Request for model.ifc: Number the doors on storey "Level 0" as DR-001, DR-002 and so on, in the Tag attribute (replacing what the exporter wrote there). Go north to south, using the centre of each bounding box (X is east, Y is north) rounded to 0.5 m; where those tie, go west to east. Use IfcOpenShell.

First a look at what the model holds.

```python
import ifcopenshell
import ifcopenshell.util.element
import ifcopenshell.util.placement

model = ifcopenshell.open("model.ifc")
print(model.schema)
storey = next(s for s in model.by_type("IfcBuildingStorey") if s.Name == "Level 0")
doors = [e for e in ifcopenshell.util.element.get_decomposition(storey) if e.is_a("IfcDoor")]
for e in sorted(doors, key=lambda e: e.id()):
    origin = ifcopenshell.util.placement.get_local_placement(e.ObjectPlacement)[:3, 3]
    print(e.id(), e.Tag, e.Name, origin.round(2) + 0.0, sep=" | ")
```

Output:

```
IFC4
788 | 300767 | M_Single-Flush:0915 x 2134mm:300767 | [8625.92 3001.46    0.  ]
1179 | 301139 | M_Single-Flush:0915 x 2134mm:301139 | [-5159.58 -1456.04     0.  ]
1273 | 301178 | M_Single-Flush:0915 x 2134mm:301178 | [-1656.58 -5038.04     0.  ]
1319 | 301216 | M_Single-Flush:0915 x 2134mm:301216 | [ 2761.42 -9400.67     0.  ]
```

```python
import ifcopenshell
import ifcopenshell.geom
import ifcopenshell.util.element
import ifcopenshell.util.shape

model = ifcopenshell.open("model.ifc")
settings = ifcopenshell.geom.settings()
settings.set("use-world-coords", True)


def centre(element):
    shape = ifcopenshell.geom.create_shape(settings, element)
    return ifcopenshell.util.shape.get_bbox_centroid(shape.geometry)


storey = next(s for s in model.by_type("IfcBuildingStorey") if s.Name == "Level 0")
doors = [e for e in ifcopenshell.util.element.get_decomposition(storey) if e.is_a("IfcDoor")]

# Insertion points can sit at a corner or the storey origin, so sort by the geometry (in metres).
centres = {e: centre(e) for e in doors}
doors.sort(key=lambda e: (-round(centres[e][1] / 0.5), centres[e][0]))

for i, e in enumerate(doors, start=1):
    number = f"DR-0{i:02d}"
    e.Tag = number
    print(e.id(), number)

model.write("model_updated.ifc")
```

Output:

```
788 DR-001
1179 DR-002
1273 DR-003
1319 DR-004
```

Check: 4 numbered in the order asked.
